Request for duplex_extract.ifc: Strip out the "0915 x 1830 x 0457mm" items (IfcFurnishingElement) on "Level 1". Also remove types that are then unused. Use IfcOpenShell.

First a look at what the model holds.

```python
import ifcopenshell
import ifcopenshell.util.element

model = ifcopenshell.open("duplex_extract.ifc")
print(model.schema)
storey = next(s for s in model.by_type("IfcBuildingStorey") if s.Name == "Level 1")
furniture = [e for e in ifcopenshell.util.element.get_decomposition(storey) if e.is_a("IfcFurnishingElement")]
seen = {}
for e in furniture:
    element_type = ifcopenshell.util.element.get_type(e)
    name = element_type.Name if element_type not in (None, e) else None
    seen[name] = seen.get(name, 0) + 1
for name, count in sorted(seen.items(), key=str):
    print(count, "x", name)
```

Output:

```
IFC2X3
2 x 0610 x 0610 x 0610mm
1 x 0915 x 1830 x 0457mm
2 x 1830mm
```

```python
import ifcopenshell
import ifcopenshell.api.root
import ifcopenshell.util.element

model = ifcopenshell.open("duplex_extract.ifc")

storey = next(s for s in model.by_type("IfcBuildingStorey") if s.Name == "Level 1")
furniture = [e for e in ifcopenshell.util.element.get_decomposition(storey) if e.is_a("IfcFurnishingElement")]
targets = [e for e in furniture if (t := ifcopenshell.util.element.get_type(e)) not in (None, e) and t.Name == "0915 x 1830 x 0457mm"]
types = {ifcopenshell.util.element.get_type(e) for e in targets} - {None, *targets}

for e in targets:
    ifcopenshell.api.root.remove_product(model, product=e)
print(len(targets), "removed")

unused = [t for t in types if not ifcopenshell.util.element.get_types(t)]
for t in unused:
    ifcopenshell.api.root.remove_product(model, product=t)
print(len(unused), "unused types removed")

model.write("duplex_extract-out.ifc")
```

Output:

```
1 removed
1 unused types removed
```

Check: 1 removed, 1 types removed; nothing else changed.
